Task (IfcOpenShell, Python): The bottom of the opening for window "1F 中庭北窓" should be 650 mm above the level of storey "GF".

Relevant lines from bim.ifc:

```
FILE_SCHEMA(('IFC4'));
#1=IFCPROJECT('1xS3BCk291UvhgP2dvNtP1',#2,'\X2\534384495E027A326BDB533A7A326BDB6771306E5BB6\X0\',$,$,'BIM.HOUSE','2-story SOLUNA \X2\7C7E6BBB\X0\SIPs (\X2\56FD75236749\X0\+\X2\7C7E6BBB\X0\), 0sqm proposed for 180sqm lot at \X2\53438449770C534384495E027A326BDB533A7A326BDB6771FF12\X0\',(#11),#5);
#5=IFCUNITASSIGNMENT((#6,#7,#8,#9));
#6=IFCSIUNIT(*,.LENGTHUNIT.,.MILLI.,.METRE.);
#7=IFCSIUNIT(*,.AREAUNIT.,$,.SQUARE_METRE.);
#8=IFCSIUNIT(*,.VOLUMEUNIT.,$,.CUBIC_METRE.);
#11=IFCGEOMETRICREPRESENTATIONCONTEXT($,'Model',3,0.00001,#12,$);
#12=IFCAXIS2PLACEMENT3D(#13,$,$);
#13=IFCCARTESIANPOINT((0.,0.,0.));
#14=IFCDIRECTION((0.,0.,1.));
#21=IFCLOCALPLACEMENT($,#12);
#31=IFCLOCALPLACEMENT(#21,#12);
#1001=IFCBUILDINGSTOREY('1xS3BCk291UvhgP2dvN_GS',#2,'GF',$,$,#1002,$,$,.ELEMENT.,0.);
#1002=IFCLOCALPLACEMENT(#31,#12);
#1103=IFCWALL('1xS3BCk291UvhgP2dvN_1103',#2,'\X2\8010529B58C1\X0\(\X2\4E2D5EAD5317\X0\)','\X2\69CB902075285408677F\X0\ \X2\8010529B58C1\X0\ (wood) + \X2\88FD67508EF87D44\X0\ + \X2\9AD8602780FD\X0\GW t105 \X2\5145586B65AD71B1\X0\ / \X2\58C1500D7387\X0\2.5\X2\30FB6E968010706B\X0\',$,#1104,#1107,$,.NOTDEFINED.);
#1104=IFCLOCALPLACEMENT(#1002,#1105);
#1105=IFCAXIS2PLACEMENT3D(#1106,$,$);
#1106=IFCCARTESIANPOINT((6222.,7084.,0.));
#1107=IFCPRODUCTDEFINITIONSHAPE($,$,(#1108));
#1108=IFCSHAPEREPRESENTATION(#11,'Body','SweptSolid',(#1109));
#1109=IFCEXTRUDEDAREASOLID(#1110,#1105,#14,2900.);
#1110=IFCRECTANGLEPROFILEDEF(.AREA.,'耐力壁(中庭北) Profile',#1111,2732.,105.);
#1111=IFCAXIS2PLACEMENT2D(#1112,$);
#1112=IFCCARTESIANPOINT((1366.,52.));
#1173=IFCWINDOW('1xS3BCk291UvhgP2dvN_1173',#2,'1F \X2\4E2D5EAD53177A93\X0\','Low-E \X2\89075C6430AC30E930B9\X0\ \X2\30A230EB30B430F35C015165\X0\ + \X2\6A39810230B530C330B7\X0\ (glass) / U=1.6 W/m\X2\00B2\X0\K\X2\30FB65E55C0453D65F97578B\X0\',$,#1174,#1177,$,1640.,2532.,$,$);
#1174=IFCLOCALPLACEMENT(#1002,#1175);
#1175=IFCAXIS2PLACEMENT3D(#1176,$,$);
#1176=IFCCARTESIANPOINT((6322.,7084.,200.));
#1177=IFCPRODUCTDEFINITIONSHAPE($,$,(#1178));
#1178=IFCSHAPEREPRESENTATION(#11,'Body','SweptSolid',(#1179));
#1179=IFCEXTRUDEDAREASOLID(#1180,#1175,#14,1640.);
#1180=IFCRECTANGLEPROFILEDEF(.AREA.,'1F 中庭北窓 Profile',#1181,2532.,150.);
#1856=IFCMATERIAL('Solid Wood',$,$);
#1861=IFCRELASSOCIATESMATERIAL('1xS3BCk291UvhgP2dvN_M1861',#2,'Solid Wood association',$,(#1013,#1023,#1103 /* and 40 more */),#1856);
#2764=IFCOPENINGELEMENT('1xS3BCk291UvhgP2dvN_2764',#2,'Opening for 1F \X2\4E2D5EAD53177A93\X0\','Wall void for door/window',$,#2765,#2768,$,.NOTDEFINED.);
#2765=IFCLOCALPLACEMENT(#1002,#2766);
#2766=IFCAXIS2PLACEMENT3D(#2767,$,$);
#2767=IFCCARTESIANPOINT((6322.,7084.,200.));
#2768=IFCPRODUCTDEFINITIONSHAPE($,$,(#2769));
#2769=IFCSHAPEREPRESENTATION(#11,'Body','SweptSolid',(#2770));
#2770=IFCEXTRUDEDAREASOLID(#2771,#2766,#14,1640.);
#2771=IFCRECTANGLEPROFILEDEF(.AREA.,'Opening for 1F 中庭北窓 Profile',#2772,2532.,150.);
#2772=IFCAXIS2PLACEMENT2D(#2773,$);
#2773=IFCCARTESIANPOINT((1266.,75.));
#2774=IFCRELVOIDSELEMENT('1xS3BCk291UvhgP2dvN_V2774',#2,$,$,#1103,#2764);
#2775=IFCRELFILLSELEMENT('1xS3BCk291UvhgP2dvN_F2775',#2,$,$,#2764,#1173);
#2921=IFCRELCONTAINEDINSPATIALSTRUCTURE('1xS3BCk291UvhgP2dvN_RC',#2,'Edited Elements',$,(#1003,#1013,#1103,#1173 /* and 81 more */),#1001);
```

```python
import numpy as np
import ifcopenshell
import ifcopenshell.api.geometry
import ifcopenshell.geom
import ifcopenshell.util.element
import ifcopenshell.util.placement
import ifcopenshell.util.shape
import ifcopenshell.util.unit

model = ifcopenshell.open("bim.ifc")
unit_scale = ifcopenshell.util.unit.calculate_unit_scale(model)

window = model.by_guid("1xS3BCk291UvhgP2dvN_1173")
opening = window.FillsVoids[0].RelatingOpeningElement
storey = ifcopenshell.util.element.get_container(window, ifc_class="IfcBuildingStorey")
level = ifcopenshell.util.placement.get_local_placement(storey.ObjectPlacement)[2, 3]

# The opening's origin need not be at the sill, so measure its lowest point.
shape = ifcopenshell.geom.create_shape(ifcopenshell.geom.settings(), opening)
bottom = ifcopenshell.util.shape.get_shape_bottom_elevation(shape, shape.geometry) / unit_scale
dz = level + 0.65 / unit_scale - bottom

shift = np.array([0.0, 0.0, dz])
# The window is not placed relative to its opening, so move both.
for product in (opening, window):
    matrix = ifcopenshell.util.placement.get_local_placement(product.ObjectPlacement)
    matrix[:3, 3] += shift
    ifcopenshell.api.geometry.edit_object_placement(model, product=product, matrix=matrix, is_si=False)

print(f"moved by {dz * unit_scale:+.3f} m")

model.write("bim-out.ifc")
```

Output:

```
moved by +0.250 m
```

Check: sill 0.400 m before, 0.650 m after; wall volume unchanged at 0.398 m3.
